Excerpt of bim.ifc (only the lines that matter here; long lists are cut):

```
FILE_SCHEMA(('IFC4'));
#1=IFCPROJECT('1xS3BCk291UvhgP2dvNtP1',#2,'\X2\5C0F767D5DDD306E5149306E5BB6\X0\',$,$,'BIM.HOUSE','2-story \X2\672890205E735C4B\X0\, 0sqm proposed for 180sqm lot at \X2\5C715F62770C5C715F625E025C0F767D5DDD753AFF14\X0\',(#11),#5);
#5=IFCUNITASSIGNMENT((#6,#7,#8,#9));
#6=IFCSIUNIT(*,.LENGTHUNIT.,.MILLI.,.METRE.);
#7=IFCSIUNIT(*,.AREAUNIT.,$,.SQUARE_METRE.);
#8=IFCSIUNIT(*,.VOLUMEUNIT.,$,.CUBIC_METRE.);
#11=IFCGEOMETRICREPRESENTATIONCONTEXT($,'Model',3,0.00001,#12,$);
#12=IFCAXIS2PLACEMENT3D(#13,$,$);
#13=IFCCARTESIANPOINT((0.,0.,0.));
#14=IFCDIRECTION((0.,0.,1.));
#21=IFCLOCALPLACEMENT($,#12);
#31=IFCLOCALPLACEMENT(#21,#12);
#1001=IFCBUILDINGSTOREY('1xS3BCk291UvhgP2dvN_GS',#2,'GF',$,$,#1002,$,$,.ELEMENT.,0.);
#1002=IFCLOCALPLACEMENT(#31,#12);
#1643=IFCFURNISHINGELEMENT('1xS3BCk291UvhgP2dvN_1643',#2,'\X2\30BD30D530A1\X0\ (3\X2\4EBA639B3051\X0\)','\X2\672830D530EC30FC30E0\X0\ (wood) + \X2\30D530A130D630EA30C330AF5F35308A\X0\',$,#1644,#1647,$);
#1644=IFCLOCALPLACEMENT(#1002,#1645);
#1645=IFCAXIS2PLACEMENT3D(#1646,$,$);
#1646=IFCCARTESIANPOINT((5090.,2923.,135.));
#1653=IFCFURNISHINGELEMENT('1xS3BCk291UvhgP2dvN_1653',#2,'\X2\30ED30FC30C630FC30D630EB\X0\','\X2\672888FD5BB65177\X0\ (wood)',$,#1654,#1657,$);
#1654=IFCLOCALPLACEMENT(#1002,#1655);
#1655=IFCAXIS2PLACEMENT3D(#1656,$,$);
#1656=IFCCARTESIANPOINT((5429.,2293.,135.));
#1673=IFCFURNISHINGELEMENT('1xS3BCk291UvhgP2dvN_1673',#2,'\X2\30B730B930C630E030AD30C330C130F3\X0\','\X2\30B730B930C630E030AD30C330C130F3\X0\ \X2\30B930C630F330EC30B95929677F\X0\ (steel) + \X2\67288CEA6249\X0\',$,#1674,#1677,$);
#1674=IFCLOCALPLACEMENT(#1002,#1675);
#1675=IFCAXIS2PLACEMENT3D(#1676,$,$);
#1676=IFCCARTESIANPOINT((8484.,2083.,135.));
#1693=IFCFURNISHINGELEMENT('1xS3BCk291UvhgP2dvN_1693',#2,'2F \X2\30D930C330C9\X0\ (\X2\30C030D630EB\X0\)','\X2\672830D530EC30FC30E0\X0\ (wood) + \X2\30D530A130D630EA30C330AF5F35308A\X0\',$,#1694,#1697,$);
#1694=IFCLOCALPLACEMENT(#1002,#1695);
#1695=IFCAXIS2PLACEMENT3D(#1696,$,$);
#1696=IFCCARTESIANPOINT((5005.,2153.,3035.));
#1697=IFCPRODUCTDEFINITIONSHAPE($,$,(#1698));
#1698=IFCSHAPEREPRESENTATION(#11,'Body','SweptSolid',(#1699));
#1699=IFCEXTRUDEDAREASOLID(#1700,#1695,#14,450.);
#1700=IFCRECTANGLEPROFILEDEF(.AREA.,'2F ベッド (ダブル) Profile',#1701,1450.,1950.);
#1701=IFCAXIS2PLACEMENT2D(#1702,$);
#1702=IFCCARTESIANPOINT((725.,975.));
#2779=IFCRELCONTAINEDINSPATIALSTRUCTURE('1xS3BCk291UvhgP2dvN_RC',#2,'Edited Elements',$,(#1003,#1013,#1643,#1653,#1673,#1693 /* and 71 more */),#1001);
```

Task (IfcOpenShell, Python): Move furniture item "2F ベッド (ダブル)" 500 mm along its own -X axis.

```python
import ifcopenshell
import ifcopenshell.api.geometry
import ifcopenshell.util.placement
import ifcopenshell.util.unit

model = ifcopenshell.open("bim.ifc")
unit_scale = ifcopenshell.util.unit.calculate_unit_scale(model)

item = model.by_id(1693)
matrix = ifcopenshell.util.placement.get_local_placement(item.ObjectPlacement)
matrix[:3, 3] -= matrix[:3, 0] * 0.5 / unit_scale
ifcopenshell.api.geometry.edit_object_placement(model, product=item, matrix=matrix, is_si=False)

print(ifcopenshell.util.placement.get_local_placement(item.ObjectPlacement).round(3) + 0.0)

model.write("bim_edited.ifc")
```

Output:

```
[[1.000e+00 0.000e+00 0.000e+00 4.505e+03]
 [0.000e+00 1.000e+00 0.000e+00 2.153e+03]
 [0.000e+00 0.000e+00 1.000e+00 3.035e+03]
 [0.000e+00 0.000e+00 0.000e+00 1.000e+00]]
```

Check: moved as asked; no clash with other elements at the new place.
